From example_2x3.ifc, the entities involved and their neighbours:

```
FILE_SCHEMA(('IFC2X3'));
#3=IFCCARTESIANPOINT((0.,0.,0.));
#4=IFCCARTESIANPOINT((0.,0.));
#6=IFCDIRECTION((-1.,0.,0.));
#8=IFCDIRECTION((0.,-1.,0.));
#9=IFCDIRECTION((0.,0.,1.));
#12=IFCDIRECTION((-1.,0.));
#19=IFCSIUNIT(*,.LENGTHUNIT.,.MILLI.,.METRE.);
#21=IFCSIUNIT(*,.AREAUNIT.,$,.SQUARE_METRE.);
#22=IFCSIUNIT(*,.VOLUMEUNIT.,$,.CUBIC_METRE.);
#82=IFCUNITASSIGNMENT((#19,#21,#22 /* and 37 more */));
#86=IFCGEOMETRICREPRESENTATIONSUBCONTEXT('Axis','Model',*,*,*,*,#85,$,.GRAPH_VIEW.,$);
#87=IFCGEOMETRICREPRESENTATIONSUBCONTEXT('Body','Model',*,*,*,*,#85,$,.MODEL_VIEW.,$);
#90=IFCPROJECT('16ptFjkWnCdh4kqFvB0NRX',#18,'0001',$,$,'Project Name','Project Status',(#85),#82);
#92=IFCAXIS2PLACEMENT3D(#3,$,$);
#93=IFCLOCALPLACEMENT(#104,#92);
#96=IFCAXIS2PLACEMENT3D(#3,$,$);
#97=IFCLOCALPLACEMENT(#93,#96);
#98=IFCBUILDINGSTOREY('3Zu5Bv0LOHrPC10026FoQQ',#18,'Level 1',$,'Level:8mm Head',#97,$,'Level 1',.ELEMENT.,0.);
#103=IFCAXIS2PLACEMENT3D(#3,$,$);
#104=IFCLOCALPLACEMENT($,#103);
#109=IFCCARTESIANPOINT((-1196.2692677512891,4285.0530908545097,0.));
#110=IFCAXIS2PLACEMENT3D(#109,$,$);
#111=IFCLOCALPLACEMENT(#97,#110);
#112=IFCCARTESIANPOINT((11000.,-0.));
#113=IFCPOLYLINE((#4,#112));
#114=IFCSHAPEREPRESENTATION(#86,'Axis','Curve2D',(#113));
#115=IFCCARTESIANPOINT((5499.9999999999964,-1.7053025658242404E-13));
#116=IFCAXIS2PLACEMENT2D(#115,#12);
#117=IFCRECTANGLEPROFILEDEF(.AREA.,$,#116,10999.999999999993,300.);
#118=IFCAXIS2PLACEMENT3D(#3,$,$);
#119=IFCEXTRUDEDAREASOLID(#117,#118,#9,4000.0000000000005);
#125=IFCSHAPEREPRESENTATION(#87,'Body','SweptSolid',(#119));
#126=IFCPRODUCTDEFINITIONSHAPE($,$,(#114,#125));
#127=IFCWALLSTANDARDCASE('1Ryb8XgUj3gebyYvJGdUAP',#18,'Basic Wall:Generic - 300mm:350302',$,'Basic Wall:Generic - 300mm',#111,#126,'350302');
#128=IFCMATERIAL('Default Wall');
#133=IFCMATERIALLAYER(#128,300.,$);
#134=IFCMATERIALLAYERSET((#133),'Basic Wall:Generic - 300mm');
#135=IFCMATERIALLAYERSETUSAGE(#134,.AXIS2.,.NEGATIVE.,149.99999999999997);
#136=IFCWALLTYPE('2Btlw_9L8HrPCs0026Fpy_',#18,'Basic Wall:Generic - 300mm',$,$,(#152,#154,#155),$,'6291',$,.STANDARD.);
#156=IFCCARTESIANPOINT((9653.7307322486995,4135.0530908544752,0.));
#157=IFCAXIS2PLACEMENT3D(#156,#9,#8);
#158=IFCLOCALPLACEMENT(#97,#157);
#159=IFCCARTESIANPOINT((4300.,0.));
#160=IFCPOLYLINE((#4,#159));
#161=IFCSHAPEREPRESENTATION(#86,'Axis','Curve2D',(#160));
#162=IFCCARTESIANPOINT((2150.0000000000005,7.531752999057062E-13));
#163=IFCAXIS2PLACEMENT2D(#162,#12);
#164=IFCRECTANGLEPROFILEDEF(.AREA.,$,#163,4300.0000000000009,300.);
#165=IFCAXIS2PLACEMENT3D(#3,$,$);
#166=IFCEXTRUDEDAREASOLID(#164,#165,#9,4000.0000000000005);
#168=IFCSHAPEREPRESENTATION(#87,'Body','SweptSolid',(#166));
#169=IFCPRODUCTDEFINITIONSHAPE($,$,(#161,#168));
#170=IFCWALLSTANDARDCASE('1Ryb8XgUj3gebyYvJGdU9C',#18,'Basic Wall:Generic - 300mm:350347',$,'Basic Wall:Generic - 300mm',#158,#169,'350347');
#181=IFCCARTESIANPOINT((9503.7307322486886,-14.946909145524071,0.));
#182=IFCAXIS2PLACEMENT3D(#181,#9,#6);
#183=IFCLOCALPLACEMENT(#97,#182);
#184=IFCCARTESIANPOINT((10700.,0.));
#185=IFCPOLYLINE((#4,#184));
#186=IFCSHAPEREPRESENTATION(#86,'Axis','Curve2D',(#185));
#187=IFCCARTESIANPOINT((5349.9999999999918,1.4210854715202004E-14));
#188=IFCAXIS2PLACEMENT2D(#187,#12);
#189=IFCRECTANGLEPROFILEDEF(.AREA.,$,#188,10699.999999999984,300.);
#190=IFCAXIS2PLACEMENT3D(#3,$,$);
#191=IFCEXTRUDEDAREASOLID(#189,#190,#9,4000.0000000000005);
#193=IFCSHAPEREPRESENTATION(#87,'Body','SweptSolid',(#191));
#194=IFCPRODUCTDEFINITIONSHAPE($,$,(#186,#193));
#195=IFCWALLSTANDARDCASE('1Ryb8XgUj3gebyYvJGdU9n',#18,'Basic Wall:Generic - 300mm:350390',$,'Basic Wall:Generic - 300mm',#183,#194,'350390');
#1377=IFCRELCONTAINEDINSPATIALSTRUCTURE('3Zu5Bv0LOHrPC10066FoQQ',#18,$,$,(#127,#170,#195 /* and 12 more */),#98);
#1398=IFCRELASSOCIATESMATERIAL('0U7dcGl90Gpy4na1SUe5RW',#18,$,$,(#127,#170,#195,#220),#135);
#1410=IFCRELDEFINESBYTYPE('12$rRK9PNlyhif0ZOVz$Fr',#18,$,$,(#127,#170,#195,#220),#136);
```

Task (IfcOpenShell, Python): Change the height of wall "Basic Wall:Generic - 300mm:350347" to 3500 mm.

```python
import ifcopenshell
import ifcopenshell.geom
import ifcopenshell.util.representation
import ifcopenshell.util.shape
import ifcopenshell.util.unit

model = ifcopenshell.open("example_2x3.ifc")
unit_scale = ifcopenshell.util.unit.calculate_unit_scale(model)
settings = ifcopenshell.geom.settings()


def volume(element):
    """Net volume in cubic metres, openings subtracted."""
    shape = ifcopenshell.geom.create_shape(settings, element)
    return ifcopenshell.util.shape.get_volume(shape.geometry)


wall = model.by_id(170)
before = volume(wall)

body = ifcopenshell.util.representation.get_representation(wall, "Model", "Body")
solid = body.Items[0]
old_height = solid.Depth
solid.Depth = 3.5 / unit_scale
after = volume(wall)

print(f"height {old_height:g} -> {solid.Depth:g}, volume {before:.3f} -> {after:.3f} m3")

model.write("example_2x3_updated.ifc")
```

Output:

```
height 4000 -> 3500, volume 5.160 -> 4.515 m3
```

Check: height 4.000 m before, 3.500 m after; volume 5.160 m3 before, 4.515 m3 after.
